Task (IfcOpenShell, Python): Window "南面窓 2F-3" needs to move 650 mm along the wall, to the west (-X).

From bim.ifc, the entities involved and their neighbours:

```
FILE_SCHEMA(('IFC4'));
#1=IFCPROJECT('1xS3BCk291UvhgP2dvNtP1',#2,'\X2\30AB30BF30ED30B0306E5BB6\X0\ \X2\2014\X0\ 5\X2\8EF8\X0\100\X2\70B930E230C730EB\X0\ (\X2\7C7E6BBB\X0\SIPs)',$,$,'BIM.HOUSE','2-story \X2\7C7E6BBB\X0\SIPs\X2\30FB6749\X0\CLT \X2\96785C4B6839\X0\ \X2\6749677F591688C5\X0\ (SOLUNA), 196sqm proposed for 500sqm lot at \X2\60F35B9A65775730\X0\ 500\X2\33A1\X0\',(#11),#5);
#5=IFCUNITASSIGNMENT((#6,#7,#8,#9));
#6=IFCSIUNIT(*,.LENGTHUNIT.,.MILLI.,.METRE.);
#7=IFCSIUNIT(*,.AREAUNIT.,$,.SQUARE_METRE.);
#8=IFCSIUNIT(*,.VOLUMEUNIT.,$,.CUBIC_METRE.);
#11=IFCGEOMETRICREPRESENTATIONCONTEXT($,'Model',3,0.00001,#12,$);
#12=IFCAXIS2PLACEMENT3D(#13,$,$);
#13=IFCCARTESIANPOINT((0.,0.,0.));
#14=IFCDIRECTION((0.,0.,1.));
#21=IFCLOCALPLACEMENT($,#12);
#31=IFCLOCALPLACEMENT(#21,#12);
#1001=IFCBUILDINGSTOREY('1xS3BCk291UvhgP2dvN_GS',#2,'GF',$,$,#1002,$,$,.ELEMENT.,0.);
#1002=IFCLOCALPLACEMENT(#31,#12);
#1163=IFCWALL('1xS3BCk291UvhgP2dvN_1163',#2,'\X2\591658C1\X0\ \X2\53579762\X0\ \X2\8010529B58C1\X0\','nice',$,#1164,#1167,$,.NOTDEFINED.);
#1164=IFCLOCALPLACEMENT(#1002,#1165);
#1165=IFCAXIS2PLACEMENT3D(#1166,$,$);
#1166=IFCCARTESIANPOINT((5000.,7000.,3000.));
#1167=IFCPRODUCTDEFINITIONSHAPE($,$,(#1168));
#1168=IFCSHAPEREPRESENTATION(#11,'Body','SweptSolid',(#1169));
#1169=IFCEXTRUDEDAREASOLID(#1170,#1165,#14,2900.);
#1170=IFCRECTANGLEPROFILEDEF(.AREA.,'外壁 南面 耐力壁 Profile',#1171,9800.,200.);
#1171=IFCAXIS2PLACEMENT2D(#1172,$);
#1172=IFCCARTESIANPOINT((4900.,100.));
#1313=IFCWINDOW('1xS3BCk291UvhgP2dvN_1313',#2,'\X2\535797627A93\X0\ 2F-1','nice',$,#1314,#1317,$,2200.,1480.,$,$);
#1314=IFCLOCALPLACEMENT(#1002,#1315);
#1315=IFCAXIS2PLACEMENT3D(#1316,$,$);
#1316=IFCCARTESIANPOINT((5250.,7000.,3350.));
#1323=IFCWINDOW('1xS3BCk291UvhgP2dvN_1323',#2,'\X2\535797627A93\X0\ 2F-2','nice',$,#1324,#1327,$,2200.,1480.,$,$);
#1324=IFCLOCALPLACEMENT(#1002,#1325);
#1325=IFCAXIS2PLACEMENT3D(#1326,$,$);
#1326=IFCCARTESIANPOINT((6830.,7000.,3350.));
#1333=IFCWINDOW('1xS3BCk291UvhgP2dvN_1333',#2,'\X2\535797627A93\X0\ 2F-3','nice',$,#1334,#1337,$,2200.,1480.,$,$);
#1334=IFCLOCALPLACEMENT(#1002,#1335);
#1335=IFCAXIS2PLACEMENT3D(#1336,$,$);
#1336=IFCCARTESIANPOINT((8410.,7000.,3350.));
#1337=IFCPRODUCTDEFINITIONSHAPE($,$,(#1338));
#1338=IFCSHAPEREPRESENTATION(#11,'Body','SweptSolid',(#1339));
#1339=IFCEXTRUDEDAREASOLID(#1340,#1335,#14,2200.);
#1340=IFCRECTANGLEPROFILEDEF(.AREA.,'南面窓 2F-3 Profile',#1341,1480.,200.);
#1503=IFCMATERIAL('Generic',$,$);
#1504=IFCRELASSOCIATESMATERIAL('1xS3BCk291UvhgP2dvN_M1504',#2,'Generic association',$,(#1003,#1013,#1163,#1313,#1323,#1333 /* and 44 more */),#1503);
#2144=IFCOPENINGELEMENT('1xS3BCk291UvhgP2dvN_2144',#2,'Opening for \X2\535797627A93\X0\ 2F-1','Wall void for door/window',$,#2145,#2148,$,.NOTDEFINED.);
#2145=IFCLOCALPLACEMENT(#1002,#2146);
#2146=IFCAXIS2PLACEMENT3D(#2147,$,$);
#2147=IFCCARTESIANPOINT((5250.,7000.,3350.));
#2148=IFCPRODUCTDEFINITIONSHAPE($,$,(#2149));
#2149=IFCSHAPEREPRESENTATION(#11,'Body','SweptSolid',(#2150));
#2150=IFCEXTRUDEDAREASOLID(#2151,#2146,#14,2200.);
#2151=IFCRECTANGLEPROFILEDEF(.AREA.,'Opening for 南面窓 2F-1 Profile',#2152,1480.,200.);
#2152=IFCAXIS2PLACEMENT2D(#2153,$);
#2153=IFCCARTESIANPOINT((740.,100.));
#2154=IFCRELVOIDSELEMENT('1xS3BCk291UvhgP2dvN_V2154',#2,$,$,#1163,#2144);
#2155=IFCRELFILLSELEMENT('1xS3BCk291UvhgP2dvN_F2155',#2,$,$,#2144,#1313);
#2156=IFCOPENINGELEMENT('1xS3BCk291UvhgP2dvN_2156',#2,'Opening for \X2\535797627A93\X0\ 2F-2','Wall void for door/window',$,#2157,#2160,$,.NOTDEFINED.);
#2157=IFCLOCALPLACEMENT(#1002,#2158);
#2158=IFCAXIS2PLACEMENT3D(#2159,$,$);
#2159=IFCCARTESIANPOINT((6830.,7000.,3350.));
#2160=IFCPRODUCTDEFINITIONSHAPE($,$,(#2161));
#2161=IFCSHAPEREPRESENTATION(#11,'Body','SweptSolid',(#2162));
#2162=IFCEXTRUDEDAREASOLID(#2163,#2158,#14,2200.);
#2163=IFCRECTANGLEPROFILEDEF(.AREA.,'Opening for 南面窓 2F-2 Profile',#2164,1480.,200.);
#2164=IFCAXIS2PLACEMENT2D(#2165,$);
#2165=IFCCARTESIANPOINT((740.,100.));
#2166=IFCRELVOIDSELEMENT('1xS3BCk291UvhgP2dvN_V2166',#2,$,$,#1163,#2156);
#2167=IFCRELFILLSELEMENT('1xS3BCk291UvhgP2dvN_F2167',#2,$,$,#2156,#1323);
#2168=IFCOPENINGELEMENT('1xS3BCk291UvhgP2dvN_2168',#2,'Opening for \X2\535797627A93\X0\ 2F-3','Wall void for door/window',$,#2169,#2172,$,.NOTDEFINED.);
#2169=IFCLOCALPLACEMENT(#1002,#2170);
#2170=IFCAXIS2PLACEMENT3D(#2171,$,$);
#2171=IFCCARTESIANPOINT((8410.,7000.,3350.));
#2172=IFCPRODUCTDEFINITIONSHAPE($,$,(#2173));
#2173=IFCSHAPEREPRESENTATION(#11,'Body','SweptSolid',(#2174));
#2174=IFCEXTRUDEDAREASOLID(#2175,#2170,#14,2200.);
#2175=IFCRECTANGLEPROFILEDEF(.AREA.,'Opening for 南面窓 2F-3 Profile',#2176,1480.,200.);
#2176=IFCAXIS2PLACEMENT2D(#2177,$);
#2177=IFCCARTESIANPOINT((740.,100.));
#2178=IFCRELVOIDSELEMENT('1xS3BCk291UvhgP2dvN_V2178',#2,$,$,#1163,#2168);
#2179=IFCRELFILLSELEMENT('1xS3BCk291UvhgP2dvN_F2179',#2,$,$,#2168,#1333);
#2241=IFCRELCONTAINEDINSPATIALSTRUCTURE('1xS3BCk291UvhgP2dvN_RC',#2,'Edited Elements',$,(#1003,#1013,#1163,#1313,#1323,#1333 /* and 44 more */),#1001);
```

```python
import ifcopenshell
import ifcopenshell.api.geometry
import ifcopenshell.util.placement
import ifcopenshell.util.unit

model = ifcopenshell.open("bim.ifc")
unit_scale = ifcopenshell.util.unit.calculate_unit_scale(model)

window = model.by_guid("1xS3BCk291UvhgP2dvN_1333")
opening = window.FillsVoids[0].RelatingOpeningElement
wall = opening.VoidsElements[0].RelatingBuildingElement

wall_matrix = ifcopenshell.util.placement.get_local_placement(wall.ObjectPlacement)
shift = wall_matrix[:3, 0] * -0.65 / unit_scale
before = ifcopenshell.util.placement.get_local_placement(window.ObjectPlacement)[:3, 3].copy()

# The window is not placed relative to its opening, so move both.
for product in (opening, window):
    matrix = ifcopenshell.util.placement.get_local_placement(product.ObjectPlacement)
    matrix[:3, 3] += shift
    ifcopenshell.api.geometry.edit_object_placement(model, product=product, matrix=matrix, is_si=False)

after = ifcopenshell.util.placement.get_local_placement(window.ObjectPlacement)[:3, 3]
print("window moved by", (after - before).round(3) + 0.0)

model.write("bim_updated.ifc")
```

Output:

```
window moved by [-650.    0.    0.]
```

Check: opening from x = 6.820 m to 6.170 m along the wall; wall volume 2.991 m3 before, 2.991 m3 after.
